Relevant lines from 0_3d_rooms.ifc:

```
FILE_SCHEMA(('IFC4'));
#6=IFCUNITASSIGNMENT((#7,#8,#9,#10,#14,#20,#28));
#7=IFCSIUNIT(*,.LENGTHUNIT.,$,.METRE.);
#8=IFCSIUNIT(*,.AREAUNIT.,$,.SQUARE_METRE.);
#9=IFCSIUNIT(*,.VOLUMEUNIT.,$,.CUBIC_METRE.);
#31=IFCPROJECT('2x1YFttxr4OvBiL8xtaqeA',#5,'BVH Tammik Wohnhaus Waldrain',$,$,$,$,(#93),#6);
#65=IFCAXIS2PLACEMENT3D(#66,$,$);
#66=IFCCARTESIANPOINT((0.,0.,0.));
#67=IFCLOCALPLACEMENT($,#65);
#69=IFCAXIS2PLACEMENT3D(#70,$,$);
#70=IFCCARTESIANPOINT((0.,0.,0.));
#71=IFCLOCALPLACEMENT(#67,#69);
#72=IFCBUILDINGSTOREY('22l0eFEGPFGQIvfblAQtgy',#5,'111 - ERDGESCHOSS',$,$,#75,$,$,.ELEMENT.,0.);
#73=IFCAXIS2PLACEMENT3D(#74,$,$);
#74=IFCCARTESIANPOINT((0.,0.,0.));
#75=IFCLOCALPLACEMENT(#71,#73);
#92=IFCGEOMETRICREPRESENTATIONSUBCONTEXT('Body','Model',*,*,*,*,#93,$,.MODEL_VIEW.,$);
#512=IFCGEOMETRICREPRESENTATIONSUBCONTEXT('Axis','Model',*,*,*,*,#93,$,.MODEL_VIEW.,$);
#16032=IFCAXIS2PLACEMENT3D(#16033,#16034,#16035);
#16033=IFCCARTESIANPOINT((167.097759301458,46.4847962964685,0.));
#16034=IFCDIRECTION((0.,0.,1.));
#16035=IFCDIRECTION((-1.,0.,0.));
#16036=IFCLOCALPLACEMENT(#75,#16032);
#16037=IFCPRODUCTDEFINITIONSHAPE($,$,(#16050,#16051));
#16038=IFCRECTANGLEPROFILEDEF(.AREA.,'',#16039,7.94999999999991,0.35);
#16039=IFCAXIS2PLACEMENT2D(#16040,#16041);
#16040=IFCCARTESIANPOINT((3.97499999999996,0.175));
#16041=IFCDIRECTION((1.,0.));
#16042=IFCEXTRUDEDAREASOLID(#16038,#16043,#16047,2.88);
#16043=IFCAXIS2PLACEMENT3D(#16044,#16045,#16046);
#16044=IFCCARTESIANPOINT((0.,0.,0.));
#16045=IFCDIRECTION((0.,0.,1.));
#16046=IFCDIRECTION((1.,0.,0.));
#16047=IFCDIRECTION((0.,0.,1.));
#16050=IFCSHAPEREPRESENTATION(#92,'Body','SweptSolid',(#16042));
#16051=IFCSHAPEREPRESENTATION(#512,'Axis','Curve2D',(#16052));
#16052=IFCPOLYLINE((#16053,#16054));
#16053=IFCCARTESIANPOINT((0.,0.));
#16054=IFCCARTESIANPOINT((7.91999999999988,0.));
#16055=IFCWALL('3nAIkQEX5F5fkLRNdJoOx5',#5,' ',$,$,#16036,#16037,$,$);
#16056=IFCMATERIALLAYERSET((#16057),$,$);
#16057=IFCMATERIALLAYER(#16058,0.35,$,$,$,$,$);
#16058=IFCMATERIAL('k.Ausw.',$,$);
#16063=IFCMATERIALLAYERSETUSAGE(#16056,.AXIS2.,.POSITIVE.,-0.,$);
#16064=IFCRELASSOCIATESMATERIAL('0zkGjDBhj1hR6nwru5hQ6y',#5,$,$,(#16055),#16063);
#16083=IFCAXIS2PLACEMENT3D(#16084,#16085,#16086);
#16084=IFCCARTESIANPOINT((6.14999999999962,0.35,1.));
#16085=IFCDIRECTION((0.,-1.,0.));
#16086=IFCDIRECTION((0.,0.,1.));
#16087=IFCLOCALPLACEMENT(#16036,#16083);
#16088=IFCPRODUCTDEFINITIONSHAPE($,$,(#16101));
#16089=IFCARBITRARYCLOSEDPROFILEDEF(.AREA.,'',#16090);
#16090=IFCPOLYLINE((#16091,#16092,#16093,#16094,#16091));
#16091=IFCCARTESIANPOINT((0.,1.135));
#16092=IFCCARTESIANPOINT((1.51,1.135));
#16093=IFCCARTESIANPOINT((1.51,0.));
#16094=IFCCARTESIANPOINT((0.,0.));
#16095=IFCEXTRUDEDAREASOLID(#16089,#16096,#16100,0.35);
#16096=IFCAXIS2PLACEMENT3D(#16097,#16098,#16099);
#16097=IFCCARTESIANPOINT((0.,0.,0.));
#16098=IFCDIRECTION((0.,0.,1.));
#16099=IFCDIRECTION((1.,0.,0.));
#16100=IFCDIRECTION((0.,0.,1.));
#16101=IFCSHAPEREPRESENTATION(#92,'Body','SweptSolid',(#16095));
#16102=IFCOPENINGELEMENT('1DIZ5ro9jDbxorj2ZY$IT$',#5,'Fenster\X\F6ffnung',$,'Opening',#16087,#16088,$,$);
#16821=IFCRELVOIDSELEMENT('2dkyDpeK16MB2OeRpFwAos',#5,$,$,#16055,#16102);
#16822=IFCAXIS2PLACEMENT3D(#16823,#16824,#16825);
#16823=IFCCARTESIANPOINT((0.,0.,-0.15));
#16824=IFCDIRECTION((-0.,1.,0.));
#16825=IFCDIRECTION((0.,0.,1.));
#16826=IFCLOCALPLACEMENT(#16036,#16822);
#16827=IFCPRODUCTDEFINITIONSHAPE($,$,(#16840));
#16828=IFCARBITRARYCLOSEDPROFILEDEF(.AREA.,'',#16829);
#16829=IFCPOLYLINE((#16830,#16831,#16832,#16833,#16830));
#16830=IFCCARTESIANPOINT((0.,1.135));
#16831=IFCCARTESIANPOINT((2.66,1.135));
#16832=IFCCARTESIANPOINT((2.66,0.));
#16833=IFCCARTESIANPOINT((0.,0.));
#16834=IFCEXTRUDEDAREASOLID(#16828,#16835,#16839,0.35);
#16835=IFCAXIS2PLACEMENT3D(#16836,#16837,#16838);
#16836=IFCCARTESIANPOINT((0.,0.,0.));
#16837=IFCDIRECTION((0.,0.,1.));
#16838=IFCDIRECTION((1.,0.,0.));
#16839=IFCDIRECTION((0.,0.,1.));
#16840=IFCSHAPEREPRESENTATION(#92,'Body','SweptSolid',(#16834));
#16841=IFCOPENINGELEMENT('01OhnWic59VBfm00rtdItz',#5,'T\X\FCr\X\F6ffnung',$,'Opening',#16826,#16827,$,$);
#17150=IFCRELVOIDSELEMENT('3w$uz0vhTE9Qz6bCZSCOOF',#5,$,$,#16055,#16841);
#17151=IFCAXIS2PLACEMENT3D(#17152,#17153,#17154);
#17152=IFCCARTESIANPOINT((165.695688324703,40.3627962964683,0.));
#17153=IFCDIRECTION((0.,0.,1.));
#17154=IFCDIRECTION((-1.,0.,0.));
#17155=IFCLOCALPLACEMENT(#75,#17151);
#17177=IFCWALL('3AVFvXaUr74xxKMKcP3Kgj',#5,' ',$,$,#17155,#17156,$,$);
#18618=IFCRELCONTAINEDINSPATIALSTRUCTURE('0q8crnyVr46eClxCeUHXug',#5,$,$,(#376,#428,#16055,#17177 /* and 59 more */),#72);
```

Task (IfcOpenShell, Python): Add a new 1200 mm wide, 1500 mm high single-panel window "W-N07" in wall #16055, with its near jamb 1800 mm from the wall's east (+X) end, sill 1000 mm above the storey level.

```python
import numpy as np
import ifcopenshell
import ifcopenshell.api.feature
import ifcopenshell.api.geometry
import ifcopenshell.api.root
import ifcopenshell.api.spatial
import ifcopenshell.geom
import ifcopenshell.util.element
import ifcopenshell.util.placement
import ifcopenshell.util.representation
import ifcopenshell.util.shape
import ifcopenshell.util.unit

model = ifcopenshell.open("0_3d_rooms.ifc")
unit_scale = ifcopenshell.util.unit.calculate_unit_scale(model)
settings = ifcopenshell.geom.settings()


def volume(element):
    """Net volume in cubic metres, openings subtracted."""
    shape = ifcopenshell.geom.create_shape(settings, element)
    return ifcopenshell.util.shape.get_volume(shape.geometry)


wall = model.by_guid("3nAIkQEX5F5fkLRNdJoOx5")
storey = ifcopenshell.util.element.get_container(wall, ifc_class="IfcBuildingStorey")
context = ifcopenshell.util.representation.get_context(model, "Model", "Body", "MODEL_VIEW")
before = volume(wall)

width, height, from_end, sill = 1.2, 1.5, 1.8, 1  # metres

# The wall runs along its own X axis, and the end named is its -X end.
wall_shape = ifcopenshell.geom.create_shape(settings, wall)
x, y, z = ifcopenshell.util.shape.get_vertices(wall_shape.geometry).T
start = x.min() + from_end
face, thickness = float(y.min()), float(y.max() - y.min())
wall_matrix = ifcopenshell.util.placement.get_local_placement(wall.ObjectPlacement)
level = ifcopenshell.util.placement.get_local_placement(storey.ObjectPlacement)[2, 3]


def in_wall(x, y):
    """Placement at x, y metres in the wall's axes, at sill height."""
    matrix = wall_matrix.copy()
    matrix[:, 3] = wall_matrix @ np.array([x / unit_scale, y / unit_scale, 0.0, 1.0])
    matrix[2, 3] = level + sill / unit_scale
    return matrix


# Opening: a box that overshoots both wall faces by 50 mm.
opening = ifcopenshell.api.root.create_entity(model, ifc_class="IfcOpeningElement", predefined_type="OPENING")
box = ifcopenshell.api.geometry.add_wall_representation(
    model, context=context, length=width, height=height, thickness=thickness + 0.1
)
ifcopenshell.api.geometry.assign_representation(model, product=opening, representation=box)
ifcopenshell.api.geometry.edit_object_placement(model, product=opening, matrix=in_wall(start, face - 0.05), is_si=False)
ifcopenshell.api.feature.add_feature(model, feature=opening, element=wall)

window = ifcopenshell.api.root.create_entity(model, ifc_class="IfcWindow", name="W-N07", predefined_type="WINDOW")
window.OverallWidth, window.OverallHeight = width / unit_scale, height / unit_scale
window.PartitioningType = "SINGLE_PANEL"
body = ifcopenshell.api.geometry.add_window_representation(
    model,
    context=context,
    overall_width=window.OverallWidth,
    overall_height=window.OverallHeight,
    partition_type="SINGLE_PANEL",
)
ifcopenshell.api.geometry.assign_representation(model, product=window, representation=body)
ifcopenshell.api.spatial.assign_container(model, products=[window], relating_structure=storey)
ifcopenshell.api.feature.add_filling(model, opening=opening, element=window)

# Centre the window in the wall's thickness.
ifcopenshell.api.geometry.edit_object_placement(model, product=window, matrix=in_wall(start, face), is_si=False)
window_shape = ifcopenshell.geom.create_shape(settings, window)
depth = ifcopenshell.util.shape.get_vertices(window_shape.geometry)[:, 1]
offset = face + thickness / 2 - (depth.min() + depth.max()) / 2
ifcopenshell.api.geometry.edit_object_placement(model, product=window, matrix=in_wall(start, offset), is_si=False)

after = volume(wall)

print(f"wall volume {before:.3f} -> {after:.3f} m3")

model.write("0_3d_rooms_edited.ifc")
```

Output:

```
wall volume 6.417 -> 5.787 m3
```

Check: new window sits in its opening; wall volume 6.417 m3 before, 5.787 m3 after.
